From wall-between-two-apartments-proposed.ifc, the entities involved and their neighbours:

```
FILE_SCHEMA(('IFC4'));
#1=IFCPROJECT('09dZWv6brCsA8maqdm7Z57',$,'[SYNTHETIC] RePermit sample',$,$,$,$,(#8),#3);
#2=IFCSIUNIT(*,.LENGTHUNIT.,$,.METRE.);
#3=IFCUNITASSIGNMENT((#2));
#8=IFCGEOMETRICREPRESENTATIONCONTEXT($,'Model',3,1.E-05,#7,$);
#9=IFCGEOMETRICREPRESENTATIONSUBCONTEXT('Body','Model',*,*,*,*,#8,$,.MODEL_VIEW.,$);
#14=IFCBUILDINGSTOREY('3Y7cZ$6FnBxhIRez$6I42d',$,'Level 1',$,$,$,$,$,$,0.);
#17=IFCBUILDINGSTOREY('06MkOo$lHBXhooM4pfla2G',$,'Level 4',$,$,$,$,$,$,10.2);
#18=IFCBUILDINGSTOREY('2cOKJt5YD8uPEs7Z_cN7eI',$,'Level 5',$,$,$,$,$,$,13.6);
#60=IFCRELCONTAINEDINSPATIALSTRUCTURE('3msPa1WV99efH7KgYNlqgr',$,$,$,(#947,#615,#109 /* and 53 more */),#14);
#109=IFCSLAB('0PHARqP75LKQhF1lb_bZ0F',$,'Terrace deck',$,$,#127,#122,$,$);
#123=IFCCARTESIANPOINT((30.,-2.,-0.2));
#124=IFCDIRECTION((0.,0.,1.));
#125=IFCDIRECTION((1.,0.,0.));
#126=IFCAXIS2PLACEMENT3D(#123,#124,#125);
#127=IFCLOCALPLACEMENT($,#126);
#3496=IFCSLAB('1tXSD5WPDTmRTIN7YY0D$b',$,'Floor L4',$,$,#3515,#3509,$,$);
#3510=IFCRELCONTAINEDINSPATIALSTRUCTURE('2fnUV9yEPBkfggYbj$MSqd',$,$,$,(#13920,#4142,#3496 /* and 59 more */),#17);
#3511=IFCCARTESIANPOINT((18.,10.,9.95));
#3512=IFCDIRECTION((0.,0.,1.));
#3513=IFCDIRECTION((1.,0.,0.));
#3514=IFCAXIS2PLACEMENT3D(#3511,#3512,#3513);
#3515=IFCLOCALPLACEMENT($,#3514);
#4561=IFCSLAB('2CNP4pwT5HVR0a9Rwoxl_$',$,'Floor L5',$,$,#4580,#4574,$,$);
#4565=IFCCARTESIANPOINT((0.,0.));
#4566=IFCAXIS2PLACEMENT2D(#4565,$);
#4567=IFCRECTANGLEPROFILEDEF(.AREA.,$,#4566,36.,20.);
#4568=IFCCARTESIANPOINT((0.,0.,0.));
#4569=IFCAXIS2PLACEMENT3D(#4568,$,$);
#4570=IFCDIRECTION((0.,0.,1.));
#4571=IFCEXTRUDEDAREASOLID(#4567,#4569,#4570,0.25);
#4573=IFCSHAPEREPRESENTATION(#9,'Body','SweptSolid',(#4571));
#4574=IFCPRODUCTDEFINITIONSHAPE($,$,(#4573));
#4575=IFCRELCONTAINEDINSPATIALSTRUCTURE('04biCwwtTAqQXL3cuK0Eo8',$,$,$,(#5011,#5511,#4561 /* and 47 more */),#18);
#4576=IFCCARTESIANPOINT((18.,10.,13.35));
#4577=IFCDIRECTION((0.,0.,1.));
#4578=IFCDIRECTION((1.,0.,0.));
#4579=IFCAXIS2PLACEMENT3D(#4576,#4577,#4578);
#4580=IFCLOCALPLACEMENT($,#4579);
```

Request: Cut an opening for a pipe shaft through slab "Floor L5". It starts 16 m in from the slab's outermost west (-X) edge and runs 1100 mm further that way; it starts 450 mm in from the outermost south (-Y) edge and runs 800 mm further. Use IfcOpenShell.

```python
import numpy as np
import ifcopenshell
import ifcopenshell.api.feature
import ifcopenshell.api.geometry
import ifcopenshell.api.root
import ifcopenshell.geom
import ifcopenshell.util.placement
import ifcopenshell.util.representation
import ifcopenshell.util.shape
import ifcopenshell.util.unit

model = ifcopenshell.open("wall-between-two-apartments-proposed.ifc")
unit_scale = ifcopenshell.util.unit.calculate_unit_scale(model)
settings = ifcopenshell.geom.settings()


def volume(element):
    """Net volume in cubic metres, openings subtracted."""
    shape = ifcopenshell.geom.create_shape(settings, element)
    return ifcopenshell.util.shape.get_volume(shape.geometry)


slab = model.by_guid("2CNP4pwT5HVR0a9Rwoxl_$")
before = volume(slab)

# Extent in the slab's own axes, in metres. The edges named are its -X and -Y sides.
slab_shape = ifcopenshell.geom.create_shape(settings, slab)
vertices = ifcopenshell.util.shape.get_vertices(slab_shape.geometry)
x_min, y_min, bottom = vertices.min(axis=0)
top = vertices[:, 2].max()

opening = ifcopenshell.api.root.create_entity(model, ifc_class="IfcOpeningElement", name="Pipe shaft opening", predefined_type="OPENING")
context = ifcopenshell.util.representation.get_context(model, "Model", "Body", "MODEL_VIEW")
width, depth = 1.1, 0.8
outline = [(0.0, 0.0), (width, 0.0), (width, depth), (0.0, depth), (0.0, 0.0)]
# Overshoot both faces by 50 mm so the cut is clean.
shape = ifcopenshell.api.geometry.add_slab_representation(
    model, context=context, depth=top - bottom + 0.1, polyline=outline
)
ifcopenshell.api.geometry.assign_representation(model, product=opening, representation=shape)

matrix = ifcopenshell.util.placement.get_local_placement(slab.ObjectPlacement)
matrix[:, 3] = matrix @ np.append(np.array([x_min + 16, y_min + 0.45, bottom - 0.05]) / unit_scale, 1.0)
ifcopenshell.api.geometry.edit_object_placement(model, product=opening, matrix=matrix, is_si=False)
ifcopenshell.api.feature.add_feature(model, feature=opening, element=slab)

after = volume(slab)

print(f"slab volume {before:.3f} -> {after:.3f} m3")

model.write("wall-between-two-apartments-proposed_updated.ifc")
```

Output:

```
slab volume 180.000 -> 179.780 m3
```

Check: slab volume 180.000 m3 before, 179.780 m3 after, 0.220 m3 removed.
